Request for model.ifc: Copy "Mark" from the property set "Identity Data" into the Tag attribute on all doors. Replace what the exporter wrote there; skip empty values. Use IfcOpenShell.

First a look at what the model holds.

```python
import ifcopenshell
import ifcopenshell.util.element

model = ifcopenshell.open("model.ifc")
print(model.schema)
doors = model.by_type("IfcDoor")
print(len(doors), "doors")
for e in doors[:8]:
    source = ifcopenshell.util.element.get_pset(e, "Identity Data", "Mark")
    target = e.Tag
    print(e.id(), repr(source), repr(target), sep=" | ")
```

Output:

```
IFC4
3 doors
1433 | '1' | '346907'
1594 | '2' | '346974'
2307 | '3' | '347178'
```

```python
import ifcopenshell
import ifcopenshell.util.element

model = ifcopenshell.open("model.ifc")

count = 0
for e in model.by_type("IfcDoor"):
    value = ifcopenshell.util.element.get_pset(e, "Identity Data", "Mark")
    current = e.Tag
    if not value or not value.strip() or current == value:
        continue
    e.Tag = value
    count += 1

print(count, "doors updated")

model.write("model_edited.ifc")
```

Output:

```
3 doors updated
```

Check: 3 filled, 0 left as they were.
